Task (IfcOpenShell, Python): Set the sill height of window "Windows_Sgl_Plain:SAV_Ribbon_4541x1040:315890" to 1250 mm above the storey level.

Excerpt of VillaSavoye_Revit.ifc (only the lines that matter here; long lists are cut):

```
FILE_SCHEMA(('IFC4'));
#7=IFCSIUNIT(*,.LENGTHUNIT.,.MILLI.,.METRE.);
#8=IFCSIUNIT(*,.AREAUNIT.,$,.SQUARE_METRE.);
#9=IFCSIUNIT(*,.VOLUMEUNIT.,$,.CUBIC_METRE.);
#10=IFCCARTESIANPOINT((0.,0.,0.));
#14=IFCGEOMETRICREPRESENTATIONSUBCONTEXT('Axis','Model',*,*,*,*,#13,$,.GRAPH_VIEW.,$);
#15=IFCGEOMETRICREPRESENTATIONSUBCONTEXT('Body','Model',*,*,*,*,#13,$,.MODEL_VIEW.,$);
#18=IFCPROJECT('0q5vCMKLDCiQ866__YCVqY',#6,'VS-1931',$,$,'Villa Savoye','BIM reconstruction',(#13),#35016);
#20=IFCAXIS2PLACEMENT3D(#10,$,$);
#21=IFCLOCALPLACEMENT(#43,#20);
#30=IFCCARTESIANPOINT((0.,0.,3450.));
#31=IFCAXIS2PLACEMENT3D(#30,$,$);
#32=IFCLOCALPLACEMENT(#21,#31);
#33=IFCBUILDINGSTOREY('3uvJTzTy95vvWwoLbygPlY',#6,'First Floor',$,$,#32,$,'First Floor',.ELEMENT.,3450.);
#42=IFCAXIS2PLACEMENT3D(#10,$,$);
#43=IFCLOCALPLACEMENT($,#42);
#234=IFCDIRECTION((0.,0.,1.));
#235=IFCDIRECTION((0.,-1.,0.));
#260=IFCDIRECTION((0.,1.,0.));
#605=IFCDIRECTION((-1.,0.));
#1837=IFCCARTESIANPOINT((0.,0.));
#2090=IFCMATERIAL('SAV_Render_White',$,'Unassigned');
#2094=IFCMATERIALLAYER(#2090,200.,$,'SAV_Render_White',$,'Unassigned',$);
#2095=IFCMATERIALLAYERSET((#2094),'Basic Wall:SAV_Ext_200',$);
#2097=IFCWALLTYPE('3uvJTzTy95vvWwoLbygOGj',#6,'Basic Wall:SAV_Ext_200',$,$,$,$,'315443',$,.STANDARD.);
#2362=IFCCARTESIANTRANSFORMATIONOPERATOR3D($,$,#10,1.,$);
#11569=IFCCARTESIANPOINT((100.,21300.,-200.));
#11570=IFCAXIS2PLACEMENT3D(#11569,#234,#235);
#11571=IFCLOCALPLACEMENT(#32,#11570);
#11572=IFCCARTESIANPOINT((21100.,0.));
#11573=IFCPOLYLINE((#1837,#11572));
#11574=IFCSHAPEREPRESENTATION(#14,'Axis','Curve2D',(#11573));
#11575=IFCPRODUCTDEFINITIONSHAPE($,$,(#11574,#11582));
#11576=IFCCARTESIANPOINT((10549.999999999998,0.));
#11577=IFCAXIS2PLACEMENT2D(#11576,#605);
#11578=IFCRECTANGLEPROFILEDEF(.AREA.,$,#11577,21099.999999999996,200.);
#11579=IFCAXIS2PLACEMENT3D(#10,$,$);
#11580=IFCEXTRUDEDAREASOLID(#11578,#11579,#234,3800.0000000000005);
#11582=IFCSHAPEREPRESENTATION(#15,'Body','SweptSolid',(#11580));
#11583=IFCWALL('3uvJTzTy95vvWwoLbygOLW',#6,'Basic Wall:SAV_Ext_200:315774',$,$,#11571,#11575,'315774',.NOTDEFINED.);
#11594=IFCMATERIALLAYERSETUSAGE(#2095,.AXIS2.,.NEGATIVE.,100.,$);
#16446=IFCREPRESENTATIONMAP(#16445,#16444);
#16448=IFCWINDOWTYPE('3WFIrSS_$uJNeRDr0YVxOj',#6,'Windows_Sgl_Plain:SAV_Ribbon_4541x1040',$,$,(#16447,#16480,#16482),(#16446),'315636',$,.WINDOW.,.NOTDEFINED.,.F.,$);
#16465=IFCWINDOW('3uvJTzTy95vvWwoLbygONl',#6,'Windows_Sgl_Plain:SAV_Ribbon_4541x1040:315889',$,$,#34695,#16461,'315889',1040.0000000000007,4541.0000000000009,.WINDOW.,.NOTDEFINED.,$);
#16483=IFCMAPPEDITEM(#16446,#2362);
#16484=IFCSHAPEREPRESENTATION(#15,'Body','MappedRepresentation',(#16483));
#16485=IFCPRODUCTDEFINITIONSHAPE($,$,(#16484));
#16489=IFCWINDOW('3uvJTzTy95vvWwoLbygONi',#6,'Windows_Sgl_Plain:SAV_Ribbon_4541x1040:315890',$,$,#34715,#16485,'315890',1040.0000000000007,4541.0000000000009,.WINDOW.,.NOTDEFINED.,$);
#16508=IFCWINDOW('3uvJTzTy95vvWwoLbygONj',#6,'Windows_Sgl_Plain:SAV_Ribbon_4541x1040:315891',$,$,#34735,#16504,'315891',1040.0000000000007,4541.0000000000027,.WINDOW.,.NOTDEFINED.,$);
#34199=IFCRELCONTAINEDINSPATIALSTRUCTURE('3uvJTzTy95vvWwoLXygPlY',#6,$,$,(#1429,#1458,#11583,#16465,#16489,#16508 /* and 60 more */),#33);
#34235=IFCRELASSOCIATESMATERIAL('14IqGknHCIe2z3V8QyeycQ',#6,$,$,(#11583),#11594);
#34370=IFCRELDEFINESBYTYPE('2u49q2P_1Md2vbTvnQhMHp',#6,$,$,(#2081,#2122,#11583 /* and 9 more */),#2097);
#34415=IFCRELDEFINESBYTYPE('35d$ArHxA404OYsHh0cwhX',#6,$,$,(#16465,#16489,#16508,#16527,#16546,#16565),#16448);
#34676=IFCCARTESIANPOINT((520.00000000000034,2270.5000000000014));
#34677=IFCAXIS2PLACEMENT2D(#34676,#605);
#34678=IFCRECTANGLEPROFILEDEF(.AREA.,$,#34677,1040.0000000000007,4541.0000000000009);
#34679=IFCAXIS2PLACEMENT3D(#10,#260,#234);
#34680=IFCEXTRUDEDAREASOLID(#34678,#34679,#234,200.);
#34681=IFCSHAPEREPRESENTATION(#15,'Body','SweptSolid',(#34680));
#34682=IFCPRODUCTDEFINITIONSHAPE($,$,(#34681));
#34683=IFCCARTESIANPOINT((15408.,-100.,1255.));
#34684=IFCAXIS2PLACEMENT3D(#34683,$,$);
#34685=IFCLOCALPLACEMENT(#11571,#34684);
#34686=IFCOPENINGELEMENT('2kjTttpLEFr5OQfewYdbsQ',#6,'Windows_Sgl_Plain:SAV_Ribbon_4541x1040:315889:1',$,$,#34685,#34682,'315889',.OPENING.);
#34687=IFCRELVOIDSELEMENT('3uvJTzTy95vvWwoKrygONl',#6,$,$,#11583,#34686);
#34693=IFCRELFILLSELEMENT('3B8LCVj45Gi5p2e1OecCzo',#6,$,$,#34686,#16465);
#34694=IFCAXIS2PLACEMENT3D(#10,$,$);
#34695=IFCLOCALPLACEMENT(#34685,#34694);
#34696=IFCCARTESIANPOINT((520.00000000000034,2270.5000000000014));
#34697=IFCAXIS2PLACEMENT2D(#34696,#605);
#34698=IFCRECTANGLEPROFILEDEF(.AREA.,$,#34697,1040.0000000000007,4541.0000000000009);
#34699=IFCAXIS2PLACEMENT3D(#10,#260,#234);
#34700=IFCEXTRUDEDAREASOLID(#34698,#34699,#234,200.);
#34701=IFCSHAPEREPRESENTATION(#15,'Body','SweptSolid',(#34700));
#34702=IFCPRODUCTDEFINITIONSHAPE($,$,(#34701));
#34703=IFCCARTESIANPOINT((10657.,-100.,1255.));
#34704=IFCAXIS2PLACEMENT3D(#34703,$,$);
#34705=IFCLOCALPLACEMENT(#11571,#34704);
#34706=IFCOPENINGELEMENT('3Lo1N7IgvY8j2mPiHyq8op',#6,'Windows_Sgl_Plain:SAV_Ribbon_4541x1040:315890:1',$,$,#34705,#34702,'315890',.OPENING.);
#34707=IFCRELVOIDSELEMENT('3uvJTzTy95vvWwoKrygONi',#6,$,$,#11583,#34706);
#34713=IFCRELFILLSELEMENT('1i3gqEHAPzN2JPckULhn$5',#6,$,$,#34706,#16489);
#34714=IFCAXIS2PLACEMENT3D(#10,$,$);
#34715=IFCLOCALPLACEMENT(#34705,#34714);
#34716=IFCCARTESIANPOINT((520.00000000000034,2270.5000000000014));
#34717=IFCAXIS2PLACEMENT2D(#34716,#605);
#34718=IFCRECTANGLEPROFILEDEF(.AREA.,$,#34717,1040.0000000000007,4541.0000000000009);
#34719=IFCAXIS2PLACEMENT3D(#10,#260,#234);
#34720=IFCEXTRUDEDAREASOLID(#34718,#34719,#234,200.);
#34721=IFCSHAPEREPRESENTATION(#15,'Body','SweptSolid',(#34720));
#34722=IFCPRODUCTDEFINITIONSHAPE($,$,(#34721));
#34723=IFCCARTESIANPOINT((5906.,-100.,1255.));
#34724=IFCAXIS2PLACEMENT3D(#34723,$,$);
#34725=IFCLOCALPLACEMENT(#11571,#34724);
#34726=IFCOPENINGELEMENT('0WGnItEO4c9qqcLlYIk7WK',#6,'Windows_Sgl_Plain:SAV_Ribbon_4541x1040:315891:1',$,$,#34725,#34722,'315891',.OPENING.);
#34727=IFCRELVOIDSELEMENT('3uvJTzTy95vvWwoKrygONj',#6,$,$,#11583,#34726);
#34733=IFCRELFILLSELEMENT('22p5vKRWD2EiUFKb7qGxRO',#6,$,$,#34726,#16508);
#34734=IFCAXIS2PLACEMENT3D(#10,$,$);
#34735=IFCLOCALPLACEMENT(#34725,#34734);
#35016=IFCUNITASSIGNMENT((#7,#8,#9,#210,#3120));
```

```python
import numpy as np
import ifcopenshell
import ifcopenshell.api.geometry
import ifcopenshell.geom
import ifcopenshell.util.element
import ifcopenshell.util.placement
import ifcopenshell.util.shape
import ifcopenshell.util.unit

model = ifcopenshell.open("VillaSavoye_Revit.ifc")
unit_scale = ifcopenshell.util.unit.calculate_unit_scale(model)

window = model.by_guid("3uvJTzTy95vvWwoLbygONi")
opening = window.FillsVoids[0].RelatingOpeningElement
storey = ifcopenshell.util.element.get_container(window, ifc_class="IfcBuildingStorey")
level = ifcopenshell.util.placement.get_local_placement(storey.ObjectPlacement)[2, 3]

# The opening's origin need not be at the sill, so measure its lowest point.
shape = ifcopenshell.geom.create_shape(ifcopenshell.geom.settings(), opening)
bottom = ifcopenshell.util.shape.get_shape_bottom_elevation(shape, shape.geometry) / unit_scale
dz = level + 1.25 / unit_scale - bottom

shift = np.array([0.0, 0.0, dz])
# The window is placed relative to its opening, so it follows when the opening moves.
matrix = ifcopenshell.util.placement.get_local_placement(opening.ObjectPlacement)
matrix[:3, 3] += shift
ifcopenshell.api.geometry.edit_object_placement(
    model, product=opening, matrix=matrix, is_si=False, should_transform_children=True
)

print(f"moved by {dz * unit_scale:+.3f} m")

model.write("VillaSavoye_Revit-out.ifc")
```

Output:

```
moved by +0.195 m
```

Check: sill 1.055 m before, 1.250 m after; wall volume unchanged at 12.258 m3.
